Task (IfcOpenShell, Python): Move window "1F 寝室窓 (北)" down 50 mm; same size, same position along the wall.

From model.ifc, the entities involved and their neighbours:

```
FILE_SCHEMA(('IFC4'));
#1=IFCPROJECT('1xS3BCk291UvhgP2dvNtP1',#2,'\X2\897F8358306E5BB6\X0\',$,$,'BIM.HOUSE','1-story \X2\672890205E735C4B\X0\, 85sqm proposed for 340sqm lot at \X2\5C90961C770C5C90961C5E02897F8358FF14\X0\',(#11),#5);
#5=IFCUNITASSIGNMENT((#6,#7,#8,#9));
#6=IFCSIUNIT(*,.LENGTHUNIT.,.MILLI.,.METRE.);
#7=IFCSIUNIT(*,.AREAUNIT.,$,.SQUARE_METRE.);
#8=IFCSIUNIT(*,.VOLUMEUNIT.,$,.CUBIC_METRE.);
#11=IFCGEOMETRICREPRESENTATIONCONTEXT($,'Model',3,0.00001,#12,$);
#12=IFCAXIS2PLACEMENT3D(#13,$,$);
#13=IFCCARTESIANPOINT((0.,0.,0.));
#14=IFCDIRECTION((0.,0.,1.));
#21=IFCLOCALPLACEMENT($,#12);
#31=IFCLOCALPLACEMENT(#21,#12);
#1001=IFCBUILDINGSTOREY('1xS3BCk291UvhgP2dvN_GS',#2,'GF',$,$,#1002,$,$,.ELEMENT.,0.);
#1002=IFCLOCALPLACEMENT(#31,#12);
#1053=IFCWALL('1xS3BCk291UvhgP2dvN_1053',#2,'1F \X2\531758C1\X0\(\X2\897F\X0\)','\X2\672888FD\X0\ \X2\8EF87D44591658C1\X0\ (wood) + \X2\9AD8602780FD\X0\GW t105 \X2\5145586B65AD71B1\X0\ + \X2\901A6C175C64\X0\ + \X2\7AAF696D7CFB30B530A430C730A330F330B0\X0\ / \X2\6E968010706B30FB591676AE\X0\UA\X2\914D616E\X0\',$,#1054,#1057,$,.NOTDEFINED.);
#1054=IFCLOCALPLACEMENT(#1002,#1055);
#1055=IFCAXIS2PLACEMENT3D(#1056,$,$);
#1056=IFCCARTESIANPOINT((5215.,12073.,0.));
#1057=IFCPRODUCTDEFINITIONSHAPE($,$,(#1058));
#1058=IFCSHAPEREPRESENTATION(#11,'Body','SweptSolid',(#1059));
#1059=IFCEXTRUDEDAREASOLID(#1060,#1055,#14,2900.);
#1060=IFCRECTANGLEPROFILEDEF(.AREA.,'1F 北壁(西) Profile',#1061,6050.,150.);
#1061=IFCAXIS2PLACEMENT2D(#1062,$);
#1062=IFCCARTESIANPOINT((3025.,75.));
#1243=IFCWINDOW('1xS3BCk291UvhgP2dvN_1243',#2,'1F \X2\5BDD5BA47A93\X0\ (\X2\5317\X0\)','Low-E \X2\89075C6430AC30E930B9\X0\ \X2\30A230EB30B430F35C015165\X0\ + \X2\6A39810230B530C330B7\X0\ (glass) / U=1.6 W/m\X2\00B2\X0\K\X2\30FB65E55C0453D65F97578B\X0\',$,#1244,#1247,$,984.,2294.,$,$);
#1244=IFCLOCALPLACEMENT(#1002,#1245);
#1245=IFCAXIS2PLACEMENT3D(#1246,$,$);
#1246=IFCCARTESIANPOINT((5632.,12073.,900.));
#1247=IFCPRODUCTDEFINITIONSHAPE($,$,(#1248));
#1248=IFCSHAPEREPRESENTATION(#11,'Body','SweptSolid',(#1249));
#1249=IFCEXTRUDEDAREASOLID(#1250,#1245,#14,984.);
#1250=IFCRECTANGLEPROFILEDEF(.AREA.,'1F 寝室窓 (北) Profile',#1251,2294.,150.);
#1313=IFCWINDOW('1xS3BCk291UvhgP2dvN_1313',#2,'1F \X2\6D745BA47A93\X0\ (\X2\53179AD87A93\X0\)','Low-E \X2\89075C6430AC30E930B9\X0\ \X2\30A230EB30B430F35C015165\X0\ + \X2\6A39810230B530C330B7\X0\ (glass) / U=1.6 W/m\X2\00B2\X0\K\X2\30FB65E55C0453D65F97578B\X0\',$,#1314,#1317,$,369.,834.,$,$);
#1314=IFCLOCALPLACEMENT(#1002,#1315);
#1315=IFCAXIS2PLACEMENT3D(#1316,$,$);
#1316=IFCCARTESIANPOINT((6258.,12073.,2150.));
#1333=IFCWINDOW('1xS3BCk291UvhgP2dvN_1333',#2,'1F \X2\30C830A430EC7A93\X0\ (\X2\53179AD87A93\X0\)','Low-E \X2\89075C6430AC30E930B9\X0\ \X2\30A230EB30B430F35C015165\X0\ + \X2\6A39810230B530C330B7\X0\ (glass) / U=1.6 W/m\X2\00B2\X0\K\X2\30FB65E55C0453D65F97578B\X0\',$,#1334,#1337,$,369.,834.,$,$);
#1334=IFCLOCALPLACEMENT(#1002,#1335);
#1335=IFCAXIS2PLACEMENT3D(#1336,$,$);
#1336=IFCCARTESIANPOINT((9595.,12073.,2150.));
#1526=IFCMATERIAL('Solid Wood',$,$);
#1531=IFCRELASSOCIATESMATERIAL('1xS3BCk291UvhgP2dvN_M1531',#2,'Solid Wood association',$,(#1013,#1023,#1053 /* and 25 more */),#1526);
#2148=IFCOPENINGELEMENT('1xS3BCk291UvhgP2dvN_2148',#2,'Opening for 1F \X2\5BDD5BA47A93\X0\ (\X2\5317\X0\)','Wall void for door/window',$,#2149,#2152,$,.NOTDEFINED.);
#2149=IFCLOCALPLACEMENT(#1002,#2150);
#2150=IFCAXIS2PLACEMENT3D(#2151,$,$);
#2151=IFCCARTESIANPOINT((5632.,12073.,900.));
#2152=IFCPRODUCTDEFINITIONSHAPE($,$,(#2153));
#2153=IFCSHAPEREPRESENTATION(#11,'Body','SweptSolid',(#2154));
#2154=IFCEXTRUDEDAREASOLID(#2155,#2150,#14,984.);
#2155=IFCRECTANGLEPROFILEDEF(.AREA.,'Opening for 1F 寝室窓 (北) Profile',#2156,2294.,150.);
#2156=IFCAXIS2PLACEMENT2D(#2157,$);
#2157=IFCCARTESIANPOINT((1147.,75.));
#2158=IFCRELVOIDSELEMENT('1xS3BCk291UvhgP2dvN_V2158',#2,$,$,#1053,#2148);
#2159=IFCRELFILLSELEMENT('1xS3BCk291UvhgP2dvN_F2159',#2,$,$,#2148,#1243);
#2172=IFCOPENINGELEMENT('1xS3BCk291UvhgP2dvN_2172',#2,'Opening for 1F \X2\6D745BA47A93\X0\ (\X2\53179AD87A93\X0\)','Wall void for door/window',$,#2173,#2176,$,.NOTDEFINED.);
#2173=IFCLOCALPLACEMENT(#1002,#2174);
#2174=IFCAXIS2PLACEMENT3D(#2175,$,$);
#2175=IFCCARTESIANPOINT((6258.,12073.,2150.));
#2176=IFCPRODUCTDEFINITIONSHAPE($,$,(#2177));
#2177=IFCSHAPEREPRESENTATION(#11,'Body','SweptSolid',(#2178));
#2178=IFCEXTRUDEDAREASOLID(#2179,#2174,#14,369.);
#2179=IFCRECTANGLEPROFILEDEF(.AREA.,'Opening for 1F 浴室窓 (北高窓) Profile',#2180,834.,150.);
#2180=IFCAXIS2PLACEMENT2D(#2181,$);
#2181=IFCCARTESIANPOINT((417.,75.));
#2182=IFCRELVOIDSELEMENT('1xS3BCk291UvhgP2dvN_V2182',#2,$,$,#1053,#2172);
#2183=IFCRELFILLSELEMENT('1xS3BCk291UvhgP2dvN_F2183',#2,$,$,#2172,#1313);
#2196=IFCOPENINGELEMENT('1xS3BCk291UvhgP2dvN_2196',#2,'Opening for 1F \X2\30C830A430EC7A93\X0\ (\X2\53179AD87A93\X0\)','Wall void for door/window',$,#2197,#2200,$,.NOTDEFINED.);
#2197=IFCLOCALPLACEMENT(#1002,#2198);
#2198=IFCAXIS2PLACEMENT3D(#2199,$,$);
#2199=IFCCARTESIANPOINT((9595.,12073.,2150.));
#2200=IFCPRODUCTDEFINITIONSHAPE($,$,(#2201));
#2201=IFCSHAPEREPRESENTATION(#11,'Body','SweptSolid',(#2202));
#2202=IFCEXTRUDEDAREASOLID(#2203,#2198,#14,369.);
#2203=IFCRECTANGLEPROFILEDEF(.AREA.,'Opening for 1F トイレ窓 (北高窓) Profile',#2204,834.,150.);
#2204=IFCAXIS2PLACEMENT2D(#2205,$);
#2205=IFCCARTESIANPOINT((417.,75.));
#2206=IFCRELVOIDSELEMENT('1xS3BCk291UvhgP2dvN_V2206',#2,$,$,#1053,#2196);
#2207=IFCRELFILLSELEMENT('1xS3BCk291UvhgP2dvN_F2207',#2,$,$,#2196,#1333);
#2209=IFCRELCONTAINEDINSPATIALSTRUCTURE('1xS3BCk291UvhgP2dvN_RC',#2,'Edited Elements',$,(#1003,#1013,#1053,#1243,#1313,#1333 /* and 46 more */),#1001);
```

```python
import numpy as np
import ifcopenshell
import ifcopenshell.api.geometry
import ifcopenshell.util.placement
import ifcopenshell.util.unit

model = ifcopenshell.open("model.ifc")
unit_scale = ifcopenshell.util.unit.calculate_unit_scale(model)

window = model.by_id(1243)
opening = window.FillsVoids[0].RelatingOpeningElement
dz = -0.05 / unit_scale

shift = np.array([0.0, 0.0, dz])
# The window is not placed relative to its opening, so move both.
for product in (opening, window):
    matrix = ifcopenshell.util.placement.get_local_placement(product.ObjectPlacement)
    matrix[:3, 3] += shift
    ifcopenshell.api.geometry.edit_object_placement(model, product=product, matrix=matrix, is_si=False)

print(f"moved by {dz * unit_scale:+.3f} m")

model.write("model_updated.ifc")
```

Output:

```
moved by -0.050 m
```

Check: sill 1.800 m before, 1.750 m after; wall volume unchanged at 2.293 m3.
